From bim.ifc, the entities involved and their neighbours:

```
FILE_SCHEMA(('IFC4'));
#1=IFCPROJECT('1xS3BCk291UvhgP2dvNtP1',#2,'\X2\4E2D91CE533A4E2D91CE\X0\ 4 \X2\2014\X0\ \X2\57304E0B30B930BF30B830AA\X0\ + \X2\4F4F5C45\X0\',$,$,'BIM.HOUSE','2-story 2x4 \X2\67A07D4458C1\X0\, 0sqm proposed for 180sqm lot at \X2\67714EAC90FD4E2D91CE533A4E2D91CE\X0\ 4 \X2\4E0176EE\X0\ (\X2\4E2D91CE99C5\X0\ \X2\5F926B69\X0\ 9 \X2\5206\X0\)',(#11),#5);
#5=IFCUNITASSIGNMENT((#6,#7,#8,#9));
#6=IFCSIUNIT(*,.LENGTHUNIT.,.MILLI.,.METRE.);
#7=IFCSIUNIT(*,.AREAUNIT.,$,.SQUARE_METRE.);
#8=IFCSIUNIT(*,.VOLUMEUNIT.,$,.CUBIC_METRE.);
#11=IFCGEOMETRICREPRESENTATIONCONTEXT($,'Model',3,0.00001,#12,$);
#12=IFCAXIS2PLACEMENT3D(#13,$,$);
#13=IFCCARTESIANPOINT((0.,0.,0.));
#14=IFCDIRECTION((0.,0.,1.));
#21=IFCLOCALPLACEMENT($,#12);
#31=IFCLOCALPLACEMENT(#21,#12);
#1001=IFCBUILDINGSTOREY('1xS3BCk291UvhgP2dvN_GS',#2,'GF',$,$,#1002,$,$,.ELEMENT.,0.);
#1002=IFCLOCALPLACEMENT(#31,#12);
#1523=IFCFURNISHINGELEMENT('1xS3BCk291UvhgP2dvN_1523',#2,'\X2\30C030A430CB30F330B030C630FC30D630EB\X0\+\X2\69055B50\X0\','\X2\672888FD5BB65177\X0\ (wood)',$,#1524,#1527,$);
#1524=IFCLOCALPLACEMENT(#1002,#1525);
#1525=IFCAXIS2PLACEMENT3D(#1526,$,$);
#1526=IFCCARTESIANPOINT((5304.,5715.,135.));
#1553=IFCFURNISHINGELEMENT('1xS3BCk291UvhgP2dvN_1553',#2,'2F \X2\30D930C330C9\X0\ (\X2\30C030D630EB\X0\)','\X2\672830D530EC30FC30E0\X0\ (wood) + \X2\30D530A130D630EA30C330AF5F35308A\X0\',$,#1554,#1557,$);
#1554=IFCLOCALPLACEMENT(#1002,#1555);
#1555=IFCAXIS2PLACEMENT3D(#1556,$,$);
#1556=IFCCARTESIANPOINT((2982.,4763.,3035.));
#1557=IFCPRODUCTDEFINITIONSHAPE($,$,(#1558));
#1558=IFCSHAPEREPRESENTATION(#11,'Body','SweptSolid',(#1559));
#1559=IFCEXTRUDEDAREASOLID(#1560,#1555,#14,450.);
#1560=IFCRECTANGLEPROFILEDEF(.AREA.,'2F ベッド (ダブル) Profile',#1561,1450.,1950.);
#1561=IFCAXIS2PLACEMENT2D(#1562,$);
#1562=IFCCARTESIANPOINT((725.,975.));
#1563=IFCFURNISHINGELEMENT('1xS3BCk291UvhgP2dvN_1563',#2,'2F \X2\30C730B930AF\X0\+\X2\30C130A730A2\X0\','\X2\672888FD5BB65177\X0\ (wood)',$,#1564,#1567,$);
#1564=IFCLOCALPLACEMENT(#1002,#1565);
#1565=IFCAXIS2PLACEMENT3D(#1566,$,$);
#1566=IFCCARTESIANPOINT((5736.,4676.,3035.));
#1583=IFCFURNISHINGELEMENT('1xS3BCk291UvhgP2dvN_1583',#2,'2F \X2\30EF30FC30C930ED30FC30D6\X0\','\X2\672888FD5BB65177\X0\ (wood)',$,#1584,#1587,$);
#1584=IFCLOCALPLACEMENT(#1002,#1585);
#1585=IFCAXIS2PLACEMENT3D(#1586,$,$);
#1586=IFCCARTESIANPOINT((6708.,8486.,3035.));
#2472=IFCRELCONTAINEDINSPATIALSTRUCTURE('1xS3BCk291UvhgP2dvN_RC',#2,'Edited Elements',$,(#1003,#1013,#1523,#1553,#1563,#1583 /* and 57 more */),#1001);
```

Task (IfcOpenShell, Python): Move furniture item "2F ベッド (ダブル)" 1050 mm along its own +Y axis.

```python
import ifcopenshell
import ifcopenshell.api.geometry
import ifcopenshell.util.placement
import ifcopenshell.util.unit

model = ifcopenshell.open("bim.ifc")
unit_scale = ifcopenshell.util.unit.calculate_unit_scale(model)

item = model.by_guid("1xS3BCk291UvhgP2dvN_1553")
matrix = ifcopenshell.util.placement.get_local_placement(item.ObjectPlacement)
matrix[:3, 3] += matrix[:3, 1] * 1.05 / unit_scale
ifcopenshell.api.geometry.edit_object_placement(model, product=item, matrix=matrix, is_si=False)

print(ifcopenshell.util.placement.get_local_placement(item.ObjectPlacement).round(3) + 0.0)

model.write("bim_updated.ifc")
```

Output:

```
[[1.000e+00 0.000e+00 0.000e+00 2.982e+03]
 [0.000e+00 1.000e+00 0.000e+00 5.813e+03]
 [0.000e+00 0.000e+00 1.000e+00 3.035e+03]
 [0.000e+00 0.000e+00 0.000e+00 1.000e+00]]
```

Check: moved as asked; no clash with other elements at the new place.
